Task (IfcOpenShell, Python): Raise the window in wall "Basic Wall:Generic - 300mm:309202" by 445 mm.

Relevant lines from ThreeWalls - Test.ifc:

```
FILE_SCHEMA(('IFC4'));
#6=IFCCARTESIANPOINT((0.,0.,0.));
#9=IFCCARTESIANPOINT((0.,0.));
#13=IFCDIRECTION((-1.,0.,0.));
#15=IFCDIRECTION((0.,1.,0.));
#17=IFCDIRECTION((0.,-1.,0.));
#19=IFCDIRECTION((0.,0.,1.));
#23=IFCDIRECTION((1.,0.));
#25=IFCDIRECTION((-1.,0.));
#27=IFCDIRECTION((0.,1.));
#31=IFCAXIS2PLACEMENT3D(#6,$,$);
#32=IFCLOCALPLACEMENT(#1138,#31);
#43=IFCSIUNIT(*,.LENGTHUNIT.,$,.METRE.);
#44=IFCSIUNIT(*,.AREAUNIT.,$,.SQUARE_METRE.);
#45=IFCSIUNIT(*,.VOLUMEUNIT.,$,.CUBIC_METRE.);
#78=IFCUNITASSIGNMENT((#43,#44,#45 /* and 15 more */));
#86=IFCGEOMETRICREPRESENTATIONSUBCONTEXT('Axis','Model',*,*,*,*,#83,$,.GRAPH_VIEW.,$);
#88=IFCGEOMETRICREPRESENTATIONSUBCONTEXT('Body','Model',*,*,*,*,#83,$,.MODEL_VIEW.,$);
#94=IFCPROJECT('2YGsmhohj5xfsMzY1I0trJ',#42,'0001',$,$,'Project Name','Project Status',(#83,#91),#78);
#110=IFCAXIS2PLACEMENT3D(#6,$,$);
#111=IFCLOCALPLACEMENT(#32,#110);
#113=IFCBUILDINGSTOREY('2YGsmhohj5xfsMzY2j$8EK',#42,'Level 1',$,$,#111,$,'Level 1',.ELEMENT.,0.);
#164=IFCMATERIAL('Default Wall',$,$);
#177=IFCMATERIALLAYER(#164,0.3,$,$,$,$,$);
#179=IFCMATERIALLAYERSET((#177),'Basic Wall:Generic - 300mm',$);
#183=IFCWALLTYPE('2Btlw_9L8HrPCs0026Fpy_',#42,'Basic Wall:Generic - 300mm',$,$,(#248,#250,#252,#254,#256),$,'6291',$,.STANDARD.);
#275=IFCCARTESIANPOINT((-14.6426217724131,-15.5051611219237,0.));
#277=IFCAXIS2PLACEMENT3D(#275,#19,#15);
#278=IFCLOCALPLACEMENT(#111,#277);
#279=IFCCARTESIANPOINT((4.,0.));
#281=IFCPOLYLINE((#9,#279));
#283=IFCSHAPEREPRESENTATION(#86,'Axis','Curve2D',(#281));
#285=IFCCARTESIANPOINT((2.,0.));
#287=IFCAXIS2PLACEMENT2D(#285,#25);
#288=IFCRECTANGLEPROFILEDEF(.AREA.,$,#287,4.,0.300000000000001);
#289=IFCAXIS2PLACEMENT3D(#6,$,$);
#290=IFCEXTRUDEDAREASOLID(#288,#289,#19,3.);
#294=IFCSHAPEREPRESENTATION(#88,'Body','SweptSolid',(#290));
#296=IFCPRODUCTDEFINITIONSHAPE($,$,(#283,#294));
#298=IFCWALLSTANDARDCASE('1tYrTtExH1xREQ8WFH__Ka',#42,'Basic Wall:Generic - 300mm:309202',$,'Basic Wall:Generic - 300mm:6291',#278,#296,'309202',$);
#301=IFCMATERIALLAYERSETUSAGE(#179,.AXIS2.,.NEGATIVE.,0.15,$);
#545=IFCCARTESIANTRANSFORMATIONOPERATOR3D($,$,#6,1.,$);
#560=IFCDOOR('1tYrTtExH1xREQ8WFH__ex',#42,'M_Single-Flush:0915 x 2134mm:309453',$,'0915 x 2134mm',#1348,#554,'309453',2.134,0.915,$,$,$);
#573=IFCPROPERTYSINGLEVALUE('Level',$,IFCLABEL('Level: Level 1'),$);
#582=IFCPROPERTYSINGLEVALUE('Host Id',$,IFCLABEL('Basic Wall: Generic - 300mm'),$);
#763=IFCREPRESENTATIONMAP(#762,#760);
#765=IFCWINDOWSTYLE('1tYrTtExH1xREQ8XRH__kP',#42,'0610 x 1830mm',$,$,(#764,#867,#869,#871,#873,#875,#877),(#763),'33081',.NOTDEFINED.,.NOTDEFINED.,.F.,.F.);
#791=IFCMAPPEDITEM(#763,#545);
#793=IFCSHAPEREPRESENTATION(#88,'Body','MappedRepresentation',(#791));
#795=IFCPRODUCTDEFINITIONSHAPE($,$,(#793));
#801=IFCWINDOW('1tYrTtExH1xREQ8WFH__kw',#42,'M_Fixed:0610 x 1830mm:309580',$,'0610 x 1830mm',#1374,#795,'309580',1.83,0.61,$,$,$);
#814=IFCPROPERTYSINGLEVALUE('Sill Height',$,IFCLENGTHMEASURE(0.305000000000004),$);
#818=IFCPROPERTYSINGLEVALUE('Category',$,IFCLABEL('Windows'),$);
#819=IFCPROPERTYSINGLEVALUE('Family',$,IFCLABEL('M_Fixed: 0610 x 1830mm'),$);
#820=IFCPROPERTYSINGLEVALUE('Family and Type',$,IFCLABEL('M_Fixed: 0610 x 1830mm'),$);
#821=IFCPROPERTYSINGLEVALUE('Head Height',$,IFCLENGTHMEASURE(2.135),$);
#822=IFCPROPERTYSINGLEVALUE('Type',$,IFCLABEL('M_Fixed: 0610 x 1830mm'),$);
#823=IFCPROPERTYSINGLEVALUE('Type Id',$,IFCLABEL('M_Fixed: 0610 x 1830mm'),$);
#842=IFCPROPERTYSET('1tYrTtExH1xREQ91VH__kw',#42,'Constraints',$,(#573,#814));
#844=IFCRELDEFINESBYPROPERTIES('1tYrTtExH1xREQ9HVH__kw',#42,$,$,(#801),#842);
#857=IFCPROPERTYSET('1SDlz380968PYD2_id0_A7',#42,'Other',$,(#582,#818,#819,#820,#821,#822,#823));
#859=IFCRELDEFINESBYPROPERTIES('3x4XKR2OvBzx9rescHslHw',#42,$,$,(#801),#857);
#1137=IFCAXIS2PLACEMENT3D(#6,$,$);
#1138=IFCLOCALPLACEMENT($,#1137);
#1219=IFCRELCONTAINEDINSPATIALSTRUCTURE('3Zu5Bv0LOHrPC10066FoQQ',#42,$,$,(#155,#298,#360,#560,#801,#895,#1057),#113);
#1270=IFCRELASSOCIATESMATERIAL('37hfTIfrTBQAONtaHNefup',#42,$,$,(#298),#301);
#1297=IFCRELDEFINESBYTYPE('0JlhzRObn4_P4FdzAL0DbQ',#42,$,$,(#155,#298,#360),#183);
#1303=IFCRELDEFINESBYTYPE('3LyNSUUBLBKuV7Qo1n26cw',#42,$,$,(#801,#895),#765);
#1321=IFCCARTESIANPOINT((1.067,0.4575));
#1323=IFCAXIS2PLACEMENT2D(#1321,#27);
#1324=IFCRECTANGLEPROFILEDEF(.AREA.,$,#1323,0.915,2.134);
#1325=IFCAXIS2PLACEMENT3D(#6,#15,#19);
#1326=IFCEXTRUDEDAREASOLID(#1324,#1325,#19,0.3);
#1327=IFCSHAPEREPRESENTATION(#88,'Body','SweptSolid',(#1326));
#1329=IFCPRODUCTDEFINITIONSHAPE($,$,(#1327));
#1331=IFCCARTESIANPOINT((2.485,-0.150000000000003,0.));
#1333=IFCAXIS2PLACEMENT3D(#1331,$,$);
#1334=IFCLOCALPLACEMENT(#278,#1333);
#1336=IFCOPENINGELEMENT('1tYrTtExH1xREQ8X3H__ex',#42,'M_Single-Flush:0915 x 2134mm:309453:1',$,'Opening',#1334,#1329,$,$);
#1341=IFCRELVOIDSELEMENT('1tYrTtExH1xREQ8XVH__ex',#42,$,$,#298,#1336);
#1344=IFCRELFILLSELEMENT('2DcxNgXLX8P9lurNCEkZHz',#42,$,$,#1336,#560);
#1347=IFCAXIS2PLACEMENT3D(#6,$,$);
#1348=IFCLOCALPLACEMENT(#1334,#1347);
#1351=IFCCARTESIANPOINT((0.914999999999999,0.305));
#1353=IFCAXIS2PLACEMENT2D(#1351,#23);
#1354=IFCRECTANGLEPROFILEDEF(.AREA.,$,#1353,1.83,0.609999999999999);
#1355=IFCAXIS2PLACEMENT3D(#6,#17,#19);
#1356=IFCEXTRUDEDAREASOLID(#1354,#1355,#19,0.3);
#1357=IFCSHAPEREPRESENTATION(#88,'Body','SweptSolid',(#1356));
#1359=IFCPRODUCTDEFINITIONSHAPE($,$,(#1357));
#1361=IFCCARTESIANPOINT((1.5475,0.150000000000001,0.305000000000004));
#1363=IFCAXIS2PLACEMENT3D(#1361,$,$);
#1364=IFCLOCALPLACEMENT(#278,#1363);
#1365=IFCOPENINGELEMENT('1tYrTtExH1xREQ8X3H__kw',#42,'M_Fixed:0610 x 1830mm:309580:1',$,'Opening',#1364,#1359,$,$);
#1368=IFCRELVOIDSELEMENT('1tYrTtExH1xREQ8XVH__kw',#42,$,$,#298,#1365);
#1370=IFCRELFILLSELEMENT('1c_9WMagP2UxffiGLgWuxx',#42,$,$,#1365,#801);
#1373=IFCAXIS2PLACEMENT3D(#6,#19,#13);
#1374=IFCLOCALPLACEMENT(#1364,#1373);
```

```python
import numpy as np
import ifcopenshell
import ifcopenshell.api.geometry
import ifcopenshell.api.pset
import ifcopenshell.util.element
import ifcopenshell.util.placement
import ifcopenshell.util.unit

model = ifcopenshell.open("ThreeWalls - Test.ifc")
unit_scale = ifcopenshell.util.unit.calculate_unit_scale(model)

window = model.by_id(801)
opening = window.FillsVoids[0].RelatingOpeningElement
dz = 0.445 / unit_scale

shift = np.array([0.0, 0.0, dz])
# The window is placed relative to its opening, so it follows when the opening moves.
matrix = ifcopenshell.util.placement.get_local_placement(opening.ObjectPlacement)
matrix[:3, 3] += shift
ifcopenshell.api.geometry.edit_object_placement(
    model, product=opening, matrix=matrix, is_si=False, should_transform_children=True
)

# Keep the stored heights in step.
pset = model.by_id(ifcopenshell.util.element.get_pset(window, "Constraints", should_inherit=False)["id"])
ifcopenshell.api.pset.edit_pset(model, pset=pset, properties={
    "Sill Height": model.create_entity("IfcLengthMeasure", ifcopenshell.util.element.get_pset(window, "Constraints", "Sill Height") + dz),
})
pset = model.by_id(ifcopenshell.util.element.get_pset(window, "Other", should_inherit=False)["id"])
ifcopenshell.api.pset.edit_pset(model, pset=pset, properties={
    "Head Height": model.create_entity("IfcLengthMeasure", ifcopenshell.util.element.get_pset(window, "Other", "Head Height") + dz),
})

print(f"moved by {dz * unit_scale:+.3f} m")

model.write("ThreeWalls - Test-out.ifc")
```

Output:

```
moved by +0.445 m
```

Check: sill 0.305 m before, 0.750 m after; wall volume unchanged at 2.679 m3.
